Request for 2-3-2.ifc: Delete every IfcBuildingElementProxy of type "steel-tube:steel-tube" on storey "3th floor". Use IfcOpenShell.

First a look at what the model holds.

```python
import ifcopenshell
import ifcopenshell.util.element

model = ifcopenshell.open("2-3-2.ifc")
print(model.schema)
storey = next(s for s in model.by_type("IfcBuildingStorey") if s.Name == "3th floor")
proxies = [e for e in ifcopenshell.util.element.get_decomposition(storey) if e.is_a("IfcBuildingElementProxy")]
seen = {}
for e in proxies:
    element_type = ifcopenshell.util.element.get_type(e)
    name = element_type.Name if element_type not in (None, e) else None
    seen[name] = seen.get(name, 0) + 1
for name, count in sorted(seen.items(), key=str):
    print(count, "x", name)
```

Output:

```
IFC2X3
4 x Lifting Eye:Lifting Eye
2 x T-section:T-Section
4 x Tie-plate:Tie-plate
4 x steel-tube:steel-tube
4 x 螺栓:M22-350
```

```python
import ifcopenshell
import ifcopenshell.api.root
import ifcopenshell.util.element

model = ifcopenshell.open("2-3-2.ifc")

storey = next(s for s in model.by_type("IfcBuildingStorey") if s.Name == "3th floor")
proxies = [e for e in ifcopenshell.util.element.get_decomposition(storey) if e.is_a("IfcBuildingElementProxy")]
targets = [e for e in proxies if (t := ifcopenshell.util.element.get_type(e)) not in (None, e) and t.Name == "steel-tube:steel-tube"]

for e in targets:
    ifcopenshell.api.root.remove_product(model, product=e)
print(len(targets), "removed")

model.write("2-3-2_v2.ifc")
```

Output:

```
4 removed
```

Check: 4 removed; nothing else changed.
